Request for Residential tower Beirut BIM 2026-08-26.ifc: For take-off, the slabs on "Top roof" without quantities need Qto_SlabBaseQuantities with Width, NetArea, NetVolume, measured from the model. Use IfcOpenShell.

First a look at what the model holds.

```python
import ifcopenshell
import ifcopenshell.util.element
import ifcopenshell.util.unit

model = ifcopenshell.open("Residential tower Beirut BIM 2026-08-26.ifc")
print(model.schema)
for unit_type in ("LENGTHUNIT", "AREAUNIT", "VOLUMEUNIT"):
    print(unit_type, ifcopenshell.util.unit.calculate_unit_scale(model, unit_type))
storey = next(s for s in model.by_type("IfcBuildingStorey") if s.Name == "Top roof")
slabs = [e for e in ifcopenshell.util.element.get_decomposition(storey) if e.is_a("IfcSlab")]
for e in sorted(slabs, key=lambda e: e.id()):
    print(e.id(), e.is_a(), e.Name, list(ifcopenshell.util.element.get_psets(e, qtos_only=True)), sep=" | ")
```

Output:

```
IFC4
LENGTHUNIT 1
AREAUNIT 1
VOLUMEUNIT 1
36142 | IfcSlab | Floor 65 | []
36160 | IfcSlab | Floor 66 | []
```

```python
import ifcopenshell
import ifcopenshell.api.pset
import ifcopenshell.geom
import ifcopenshell.util.element
import ifcopenshell.util.shape
import ifcopenshell.util.unit

model = ifcopenshell.open("Residential tower Beirut BIM 2026-08-26.ifc")
unit_scale = ifcopenshell.util.unit.calculate_unit_scale(model)
area_scale = ifcopenshell.util.unit.calculate_unit_scale(model, "AREAUNIT")
volume_scale = ifcopenshell.util.unit.calculate_unit_scale(model, "VOLUMEUNIT")
settings = ifcopenshell.geom.settings()

storey = next(s for s in model.by_type("IfcBuildingStorey") if s.Name == "Top roof")
slabs = [e for e in ifcopenshell.util.element.get_decomposition(storey) if e.is_a("IfcSlab")]

for e in sorted(slabs, key=lambda e: e.id()):
    if ifcopenshell.util.element.get_psets(e, qtos_only=True, should_inherit=False):
        continue
    # Geometry comes back in metres, in the element's own axes.
    shape = ifcopenshell.geom.create_shape(settings, e)
    values = {
        "Width": ifcopenshell.util.shape.get_z(shape.geometry) / unit_scale,
        "NetArea": ifcopenshell.util.shape.get_footprint_area(shape.geometry) / area_scale,
        "NetVolume": ifcopenshell.util.shape.get_volume(shape.geometry) / volume_scale,
    }
    qto = ifcopenshell.api.pset.add_qto(model, product=e, name="Qto_SlabBaseQuantities")
    ifcopenshell.api.pset.edit_qto(model, qto=qto, properties=values)
    print(e.id(), {k: round(v, 3) for k, v in values.items()})

model.write("Residential tower Beirut BIM 2026-08-26_rev.ifc")
```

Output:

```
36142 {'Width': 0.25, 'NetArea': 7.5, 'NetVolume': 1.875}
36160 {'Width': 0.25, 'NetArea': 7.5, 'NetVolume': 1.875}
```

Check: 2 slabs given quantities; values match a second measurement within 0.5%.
